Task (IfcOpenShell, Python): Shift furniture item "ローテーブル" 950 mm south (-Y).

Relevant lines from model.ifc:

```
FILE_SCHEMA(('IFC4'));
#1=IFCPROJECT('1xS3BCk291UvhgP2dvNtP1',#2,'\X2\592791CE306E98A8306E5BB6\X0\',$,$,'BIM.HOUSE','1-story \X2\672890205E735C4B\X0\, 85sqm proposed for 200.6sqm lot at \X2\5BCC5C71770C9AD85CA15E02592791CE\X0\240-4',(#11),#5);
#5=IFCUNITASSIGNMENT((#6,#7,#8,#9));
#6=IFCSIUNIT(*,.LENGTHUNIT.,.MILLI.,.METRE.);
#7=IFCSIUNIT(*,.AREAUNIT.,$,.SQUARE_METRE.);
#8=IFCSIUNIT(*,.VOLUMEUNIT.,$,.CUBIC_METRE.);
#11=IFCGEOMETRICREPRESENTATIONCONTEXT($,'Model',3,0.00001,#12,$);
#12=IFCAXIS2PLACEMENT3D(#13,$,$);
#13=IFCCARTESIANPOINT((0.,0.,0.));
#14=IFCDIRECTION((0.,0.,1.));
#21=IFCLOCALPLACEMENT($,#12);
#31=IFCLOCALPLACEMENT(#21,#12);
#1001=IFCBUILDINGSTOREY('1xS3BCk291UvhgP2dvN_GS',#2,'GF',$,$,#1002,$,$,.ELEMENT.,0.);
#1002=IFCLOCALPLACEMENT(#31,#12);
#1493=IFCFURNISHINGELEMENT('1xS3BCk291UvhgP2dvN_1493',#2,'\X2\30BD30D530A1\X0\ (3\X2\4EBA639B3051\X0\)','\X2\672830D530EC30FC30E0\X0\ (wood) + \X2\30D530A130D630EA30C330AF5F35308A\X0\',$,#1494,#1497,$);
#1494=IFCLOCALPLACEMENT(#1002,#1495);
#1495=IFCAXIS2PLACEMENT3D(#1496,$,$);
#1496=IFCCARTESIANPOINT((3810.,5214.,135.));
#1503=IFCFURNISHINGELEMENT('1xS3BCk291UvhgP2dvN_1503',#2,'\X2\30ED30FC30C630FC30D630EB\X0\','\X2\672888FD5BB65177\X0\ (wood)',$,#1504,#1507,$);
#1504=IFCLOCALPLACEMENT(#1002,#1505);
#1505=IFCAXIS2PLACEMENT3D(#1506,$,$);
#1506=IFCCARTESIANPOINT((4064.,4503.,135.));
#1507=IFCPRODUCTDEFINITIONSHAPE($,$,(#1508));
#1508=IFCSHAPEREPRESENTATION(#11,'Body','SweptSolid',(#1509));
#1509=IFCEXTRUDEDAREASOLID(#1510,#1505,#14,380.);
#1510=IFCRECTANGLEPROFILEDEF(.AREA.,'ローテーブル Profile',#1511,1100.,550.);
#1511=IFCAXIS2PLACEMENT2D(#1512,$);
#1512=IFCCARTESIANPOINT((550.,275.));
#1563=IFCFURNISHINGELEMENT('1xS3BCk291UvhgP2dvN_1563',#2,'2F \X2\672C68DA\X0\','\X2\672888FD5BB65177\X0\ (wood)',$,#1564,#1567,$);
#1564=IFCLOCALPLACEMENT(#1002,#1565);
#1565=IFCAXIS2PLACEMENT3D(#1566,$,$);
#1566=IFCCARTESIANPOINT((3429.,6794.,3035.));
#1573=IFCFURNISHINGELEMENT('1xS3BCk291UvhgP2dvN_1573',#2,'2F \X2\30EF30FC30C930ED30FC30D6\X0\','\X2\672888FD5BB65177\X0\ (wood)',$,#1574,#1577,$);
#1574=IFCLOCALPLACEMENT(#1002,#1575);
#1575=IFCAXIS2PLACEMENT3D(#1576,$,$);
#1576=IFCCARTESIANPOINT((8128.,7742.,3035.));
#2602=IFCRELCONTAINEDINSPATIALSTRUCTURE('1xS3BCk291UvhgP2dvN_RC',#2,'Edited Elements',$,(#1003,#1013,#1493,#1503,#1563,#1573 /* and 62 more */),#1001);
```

```python
import ifcopenshell
import ifcopenshell.api.geometry
import ifcopenshell.util.placement

model = ifcopenshell.open("model.ifc")

item = model.by_guid("1xS3BCk291UvhgP2dvN_1503")
matrix = ifcopenshell.util.placement.get_local_placement(item.ObjectPlacement)
matrix[1, 3] -= 950.0
ifcopenshell.api.geometry.edit_object_placement(model, product=item, matrix=matrix, is_si=False)

print(ifcopenshell.util.placement.get_local_placement(item.ObjectPlacement).round(3) + 0.0)

model.write("model_updated.ifc")
```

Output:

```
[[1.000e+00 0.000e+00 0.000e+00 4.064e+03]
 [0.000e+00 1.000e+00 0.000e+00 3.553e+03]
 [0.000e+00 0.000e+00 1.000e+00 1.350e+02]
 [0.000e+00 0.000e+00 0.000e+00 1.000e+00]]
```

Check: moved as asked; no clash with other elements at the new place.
